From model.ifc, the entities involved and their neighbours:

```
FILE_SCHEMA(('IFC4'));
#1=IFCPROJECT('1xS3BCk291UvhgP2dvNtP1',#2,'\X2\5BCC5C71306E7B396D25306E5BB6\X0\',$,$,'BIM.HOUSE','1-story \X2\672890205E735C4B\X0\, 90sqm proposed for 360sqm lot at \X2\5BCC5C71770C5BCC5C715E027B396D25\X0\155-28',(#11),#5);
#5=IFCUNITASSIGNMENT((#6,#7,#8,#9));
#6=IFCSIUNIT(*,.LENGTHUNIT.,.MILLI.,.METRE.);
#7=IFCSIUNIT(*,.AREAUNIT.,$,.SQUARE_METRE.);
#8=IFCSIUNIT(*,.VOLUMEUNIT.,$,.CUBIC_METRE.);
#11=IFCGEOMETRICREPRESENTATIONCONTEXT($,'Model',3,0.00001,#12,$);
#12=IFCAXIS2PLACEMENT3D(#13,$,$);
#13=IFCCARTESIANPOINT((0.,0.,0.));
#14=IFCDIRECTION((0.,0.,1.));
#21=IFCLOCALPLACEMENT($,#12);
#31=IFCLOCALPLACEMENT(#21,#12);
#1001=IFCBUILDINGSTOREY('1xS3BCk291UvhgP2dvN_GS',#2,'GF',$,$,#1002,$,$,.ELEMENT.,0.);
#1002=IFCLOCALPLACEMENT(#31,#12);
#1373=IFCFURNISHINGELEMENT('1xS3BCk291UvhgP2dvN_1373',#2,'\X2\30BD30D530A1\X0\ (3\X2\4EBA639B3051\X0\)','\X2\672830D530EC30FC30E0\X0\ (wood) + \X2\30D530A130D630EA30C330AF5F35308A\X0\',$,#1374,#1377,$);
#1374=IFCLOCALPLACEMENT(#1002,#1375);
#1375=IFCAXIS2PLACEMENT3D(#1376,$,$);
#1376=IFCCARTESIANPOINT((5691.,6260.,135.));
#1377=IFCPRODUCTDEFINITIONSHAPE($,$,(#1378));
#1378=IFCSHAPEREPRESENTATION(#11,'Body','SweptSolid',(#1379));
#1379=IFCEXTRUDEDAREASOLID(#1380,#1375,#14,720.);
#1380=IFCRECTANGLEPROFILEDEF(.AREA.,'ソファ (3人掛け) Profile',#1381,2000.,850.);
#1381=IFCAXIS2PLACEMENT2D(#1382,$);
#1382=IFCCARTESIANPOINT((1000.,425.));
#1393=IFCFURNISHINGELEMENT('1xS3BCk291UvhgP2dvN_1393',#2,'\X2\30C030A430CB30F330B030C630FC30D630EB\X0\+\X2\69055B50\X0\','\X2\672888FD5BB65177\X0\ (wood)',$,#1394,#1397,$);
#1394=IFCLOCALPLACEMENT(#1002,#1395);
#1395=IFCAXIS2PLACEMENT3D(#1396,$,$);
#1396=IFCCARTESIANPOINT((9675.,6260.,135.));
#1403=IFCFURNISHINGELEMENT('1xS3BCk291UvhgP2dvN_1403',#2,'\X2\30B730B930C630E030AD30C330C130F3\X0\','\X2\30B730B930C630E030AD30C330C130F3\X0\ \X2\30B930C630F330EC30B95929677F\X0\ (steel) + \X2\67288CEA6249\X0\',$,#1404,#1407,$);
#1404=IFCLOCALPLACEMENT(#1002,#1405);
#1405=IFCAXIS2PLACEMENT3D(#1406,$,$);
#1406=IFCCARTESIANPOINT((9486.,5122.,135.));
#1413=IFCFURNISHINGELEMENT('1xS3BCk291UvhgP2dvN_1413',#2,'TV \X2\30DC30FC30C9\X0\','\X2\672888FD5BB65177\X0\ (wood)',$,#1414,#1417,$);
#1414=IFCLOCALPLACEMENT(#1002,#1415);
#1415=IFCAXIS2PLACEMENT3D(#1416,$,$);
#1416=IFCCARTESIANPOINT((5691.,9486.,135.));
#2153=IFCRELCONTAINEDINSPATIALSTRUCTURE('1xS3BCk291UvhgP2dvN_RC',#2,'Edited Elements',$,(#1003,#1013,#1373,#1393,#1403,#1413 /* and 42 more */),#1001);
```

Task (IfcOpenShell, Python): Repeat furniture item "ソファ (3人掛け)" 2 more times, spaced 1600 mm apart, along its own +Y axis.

```python
import ifcopenshell
import ifcopenshell.api.geometry
import ifcopenshell.api.root
import ifcopenshell.util.element
import ifcopenshell.util.placement
import ifcopenshell.util.unit

model = ifcopenshell.open("model.ifc")
unit_scale = ifcopenshell.util.unit.calculate_unit_scale(model)


def reuse_history(source, copy):
    """copy_class also copies each property set's owner history, people and application; keep the originals."""
    for rel in copy.IsDefinedBy:
        if rel.is_a("IfcRelDefinesByProperties") and (history := rel.RelatingPropertyDefinition.OwnerHistory):
            rel.RelatingPropertyDefinition.OwnerHistory = source.OwnerHistory
            ifcopenshell.util.element.remove_deep2(model, history)


source = model.by_guid("1xS3BCk291UvhgP2dvN_1373")
base = ifcopenshell.util.placement.get_local_placement(source.ObjectPlacement)
step = base[:3, 1] * 1.6 / unit_scale

for i in range(1, 3):
    copy = ifcopenshell.api.root.copy_class(model, product=source)
    copy.Representation = ifcopenshell.util.element.copy_deep(
        model, source.Representation, exclude=["IfcGeometricRepresentationContext", "IfcRepresentationMap"]
    )
    reuse_history(source, copy)
    matrix = base.copy()
    matrix[:3, 3] += i * step
    print("added at", matrix[:3, 3].round(3) + 0.0)
    ifcopenshell.api.geometry.edit_object_placement(model, product=copy, matrix=matrix, is_si=False)

model.write("model_rev.ifc")
```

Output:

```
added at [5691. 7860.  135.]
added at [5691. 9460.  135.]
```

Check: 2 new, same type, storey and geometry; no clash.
